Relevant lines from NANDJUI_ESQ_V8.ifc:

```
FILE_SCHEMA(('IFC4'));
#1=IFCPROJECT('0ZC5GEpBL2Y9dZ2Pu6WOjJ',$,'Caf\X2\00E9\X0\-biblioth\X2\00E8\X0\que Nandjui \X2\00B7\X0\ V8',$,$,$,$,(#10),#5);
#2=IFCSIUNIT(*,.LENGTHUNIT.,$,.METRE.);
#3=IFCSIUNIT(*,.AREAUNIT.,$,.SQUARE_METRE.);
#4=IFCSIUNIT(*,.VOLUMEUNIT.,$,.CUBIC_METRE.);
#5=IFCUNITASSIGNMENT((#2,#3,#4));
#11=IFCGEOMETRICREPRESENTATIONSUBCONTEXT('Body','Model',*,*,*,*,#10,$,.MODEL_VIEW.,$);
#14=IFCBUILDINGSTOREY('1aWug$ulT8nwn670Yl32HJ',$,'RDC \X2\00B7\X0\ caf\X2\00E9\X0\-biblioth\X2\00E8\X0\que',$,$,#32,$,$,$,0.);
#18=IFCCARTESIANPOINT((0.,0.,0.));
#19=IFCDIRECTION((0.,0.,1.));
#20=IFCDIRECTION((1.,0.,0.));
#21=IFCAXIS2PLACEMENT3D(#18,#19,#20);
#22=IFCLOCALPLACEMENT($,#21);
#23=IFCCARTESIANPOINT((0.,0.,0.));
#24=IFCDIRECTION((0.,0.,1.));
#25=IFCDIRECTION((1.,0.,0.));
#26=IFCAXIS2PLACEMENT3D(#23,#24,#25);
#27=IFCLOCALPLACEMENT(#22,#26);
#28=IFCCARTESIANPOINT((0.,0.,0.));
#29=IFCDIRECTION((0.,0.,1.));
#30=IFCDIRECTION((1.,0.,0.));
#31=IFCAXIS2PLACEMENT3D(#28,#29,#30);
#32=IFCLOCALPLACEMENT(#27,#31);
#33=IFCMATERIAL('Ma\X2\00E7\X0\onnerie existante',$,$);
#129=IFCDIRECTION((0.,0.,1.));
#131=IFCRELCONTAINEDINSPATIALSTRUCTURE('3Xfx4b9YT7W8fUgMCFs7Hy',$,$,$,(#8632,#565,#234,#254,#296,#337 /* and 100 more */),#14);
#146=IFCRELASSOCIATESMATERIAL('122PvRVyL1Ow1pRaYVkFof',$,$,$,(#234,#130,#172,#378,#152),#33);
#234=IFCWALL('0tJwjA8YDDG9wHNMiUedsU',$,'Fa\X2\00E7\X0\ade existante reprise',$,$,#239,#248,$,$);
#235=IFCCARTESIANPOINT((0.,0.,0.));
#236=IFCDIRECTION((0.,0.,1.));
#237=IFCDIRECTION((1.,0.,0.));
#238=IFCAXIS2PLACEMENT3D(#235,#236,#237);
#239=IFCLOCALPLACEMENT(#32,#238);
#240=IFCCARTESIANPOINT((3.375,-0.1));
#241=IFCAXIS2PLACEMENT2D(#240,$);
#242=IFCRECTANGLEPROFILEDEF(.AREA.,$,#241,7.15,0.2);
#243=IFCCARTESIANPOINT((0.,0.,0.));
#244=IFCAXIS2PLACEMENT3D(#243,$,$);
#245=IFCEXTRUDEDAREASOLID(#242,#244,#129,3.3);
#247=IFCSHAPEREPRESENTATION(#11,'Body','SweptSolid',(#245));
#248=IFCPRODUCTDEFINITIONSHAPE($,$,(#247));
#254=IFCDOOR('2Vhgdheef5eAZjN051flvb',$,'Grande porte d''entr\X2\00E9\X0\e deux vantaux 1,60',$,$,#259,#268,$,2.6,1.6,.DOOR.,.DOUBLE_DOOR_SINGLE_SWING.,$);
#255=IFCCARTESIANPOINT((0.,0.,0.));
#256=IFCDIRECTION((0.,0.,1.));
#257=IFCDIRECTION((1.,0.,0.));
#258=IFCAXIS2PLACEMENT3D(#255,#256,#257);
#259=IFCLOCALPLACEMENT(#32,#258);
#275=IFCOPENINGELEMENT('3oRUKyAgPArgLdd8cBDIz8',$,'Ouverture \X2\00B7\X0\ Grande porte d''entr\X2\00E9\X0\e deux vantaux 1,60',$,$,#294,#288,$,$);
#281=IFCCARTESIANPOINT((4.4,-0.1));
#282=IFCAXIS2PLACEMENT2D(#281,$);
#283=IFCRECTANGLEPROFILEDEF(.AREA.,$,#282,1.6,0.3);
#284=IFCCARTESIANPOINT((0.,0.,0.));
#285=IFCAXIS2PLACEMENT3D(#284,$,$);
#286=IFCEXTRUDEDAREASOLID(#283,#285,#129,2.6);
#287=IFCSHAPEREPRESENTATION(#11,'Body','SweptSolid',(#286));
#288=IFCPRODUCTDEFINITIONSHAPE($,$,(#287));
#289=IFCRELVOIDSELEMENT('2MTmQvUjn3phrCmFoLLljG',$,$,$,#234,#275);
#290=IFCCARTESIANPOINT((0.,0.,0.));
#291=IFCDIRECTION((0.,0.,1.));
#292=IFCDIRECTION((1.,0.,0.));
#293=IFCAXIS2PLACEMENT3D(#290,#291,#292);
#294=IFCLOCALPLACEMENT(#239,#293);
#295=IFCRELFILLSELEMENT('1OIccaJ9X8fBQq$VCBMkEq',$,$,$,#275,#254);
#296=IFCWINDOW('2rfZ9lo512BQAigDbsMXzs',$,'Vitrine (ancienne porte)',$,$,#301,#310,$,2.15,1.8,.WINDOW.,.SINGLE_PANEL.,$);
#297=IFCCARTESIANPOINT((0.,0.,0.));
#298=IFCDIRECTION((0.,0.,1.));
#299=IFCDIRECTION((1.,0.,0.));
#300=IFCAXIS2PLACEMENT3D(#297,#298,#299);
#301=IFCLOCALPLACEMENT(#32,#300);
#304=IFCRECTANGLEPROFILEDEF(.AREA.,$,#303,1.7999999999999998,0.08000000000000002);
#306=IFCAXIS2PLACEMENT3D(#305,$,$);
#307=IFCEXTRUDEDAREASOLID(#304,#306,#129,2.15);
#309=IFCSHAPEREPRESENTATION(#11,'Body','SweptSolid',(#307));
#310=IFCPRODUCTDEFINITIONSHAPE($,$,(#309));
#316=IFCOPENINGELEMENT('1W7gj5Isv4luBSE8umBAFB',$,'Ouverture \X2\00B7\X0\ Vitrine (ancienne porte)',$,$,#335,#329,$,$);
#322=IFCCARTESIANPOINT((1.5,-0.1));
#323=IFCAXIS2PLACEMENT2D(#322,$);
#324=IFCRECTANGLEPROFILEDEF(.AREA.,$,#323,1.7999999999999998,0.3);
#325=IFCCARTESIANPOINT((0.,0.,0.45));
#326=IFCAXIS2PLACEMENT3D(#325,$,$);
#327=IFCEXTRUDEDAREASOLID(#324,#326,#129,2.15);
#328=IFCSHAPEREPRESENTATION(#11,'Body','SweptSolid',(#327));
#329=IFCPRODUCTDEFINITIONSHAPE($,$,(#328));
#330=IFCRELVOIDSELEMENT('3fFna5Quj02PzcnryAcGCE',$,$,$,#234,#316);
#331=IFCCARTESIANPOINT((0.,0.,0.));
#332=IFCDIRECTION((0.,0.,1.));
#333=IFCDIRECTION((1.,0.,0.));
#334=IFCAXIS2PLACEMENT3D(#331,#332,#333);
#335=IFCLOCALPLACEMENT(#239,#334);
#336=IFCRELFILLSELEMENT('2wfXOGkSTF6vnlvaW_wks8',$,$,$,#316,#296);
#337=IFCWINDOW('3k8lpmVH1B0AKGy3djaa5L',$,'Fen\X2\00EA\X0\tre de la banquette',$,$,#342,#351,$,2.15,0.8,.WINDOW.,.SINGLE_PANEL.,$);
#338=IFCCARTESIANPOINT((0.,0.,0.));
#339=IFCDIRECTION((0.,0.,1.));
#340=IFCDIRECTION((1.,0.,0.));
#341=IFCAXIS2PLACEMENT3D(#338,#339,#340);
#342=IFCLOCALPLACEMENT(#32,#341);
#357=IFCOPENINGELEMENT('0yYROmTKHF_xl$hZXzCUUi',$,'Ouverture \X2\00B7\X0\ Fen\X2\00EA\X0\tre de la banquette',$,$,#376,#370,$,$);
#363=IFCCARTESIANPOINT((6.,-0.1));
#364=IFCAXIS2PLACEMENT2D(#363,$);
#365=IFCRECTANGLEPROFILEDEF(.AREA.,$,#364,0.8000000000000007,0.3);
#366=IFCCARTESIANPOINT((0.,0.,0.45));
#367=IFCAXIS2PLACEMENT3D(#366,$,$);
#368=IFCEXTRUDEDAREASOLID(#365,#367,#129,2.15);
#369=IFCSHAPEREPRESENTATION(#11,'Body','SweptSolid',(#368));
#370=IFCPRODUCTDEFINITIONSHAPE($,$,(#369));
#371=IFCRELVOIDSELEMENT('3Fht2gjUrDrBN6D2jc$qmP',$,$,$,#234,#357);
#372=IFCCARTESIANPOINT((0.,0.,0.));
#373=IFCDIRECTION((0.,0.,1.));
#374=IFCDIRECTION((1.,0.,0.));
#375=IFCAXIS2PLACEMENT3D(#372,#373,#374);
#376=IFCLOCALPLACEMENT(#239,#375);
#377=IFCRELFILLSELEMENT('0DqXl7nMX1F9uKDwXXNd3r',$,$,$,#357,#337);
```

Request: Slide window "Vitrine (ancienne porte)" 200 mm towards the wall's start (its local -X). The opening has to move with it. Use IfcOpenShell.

```python
import ifcopenshell
import ifcopenshell.api.geometry
import ifcopenshell.util.placement
import ifcopenshell.util.unit

model = ifcopenshell.open("NANDJUI_ESQ_V8.ifc")
unit_scale = ifcopenshell.util.unit.calculate_unit_scale(model)

window = model.by_guid("2rfZ9lo512BQAigDbsMXzs")
opening = window.FillsVoids[0].RelatingOpeningElement
wall = opening.VoidsElements[0].RelatingBuildingElement

wall_matrix = ifcopenshell.util.placement.get_local_placement(wall.ObjectPlacement)
shift = wall_matrix[:3, 0] * -0.2 / unit_scale
before = ifcopenshell.util.placement.get_local_placement(window.ObjectPlacement)[:3, 3].copy()

# The window is not placed relative to its opening, so move both.
for product in (opening, window):
    matrix = ifcopenshell.util.placement.get_local_placement(product.ObjectPlacement)
    matrix[:3, 3] += shift
    ifcopenshell.api.geometry.edit_object_placement(model, product=product, matrix=matrix, is_si=False)

after = ifcopenshell.util.placement.get_local_placement(window.ObjectPlacement)[:3, 3]
print("window moved by", (after - before).round(3) + 0.0)

model.write("NANDJUI_ESQ_V8_updated.ifc")
```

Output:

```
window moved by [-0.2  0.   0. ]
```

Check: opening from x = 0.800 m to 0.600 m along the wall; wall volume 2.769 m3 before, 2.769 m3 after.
